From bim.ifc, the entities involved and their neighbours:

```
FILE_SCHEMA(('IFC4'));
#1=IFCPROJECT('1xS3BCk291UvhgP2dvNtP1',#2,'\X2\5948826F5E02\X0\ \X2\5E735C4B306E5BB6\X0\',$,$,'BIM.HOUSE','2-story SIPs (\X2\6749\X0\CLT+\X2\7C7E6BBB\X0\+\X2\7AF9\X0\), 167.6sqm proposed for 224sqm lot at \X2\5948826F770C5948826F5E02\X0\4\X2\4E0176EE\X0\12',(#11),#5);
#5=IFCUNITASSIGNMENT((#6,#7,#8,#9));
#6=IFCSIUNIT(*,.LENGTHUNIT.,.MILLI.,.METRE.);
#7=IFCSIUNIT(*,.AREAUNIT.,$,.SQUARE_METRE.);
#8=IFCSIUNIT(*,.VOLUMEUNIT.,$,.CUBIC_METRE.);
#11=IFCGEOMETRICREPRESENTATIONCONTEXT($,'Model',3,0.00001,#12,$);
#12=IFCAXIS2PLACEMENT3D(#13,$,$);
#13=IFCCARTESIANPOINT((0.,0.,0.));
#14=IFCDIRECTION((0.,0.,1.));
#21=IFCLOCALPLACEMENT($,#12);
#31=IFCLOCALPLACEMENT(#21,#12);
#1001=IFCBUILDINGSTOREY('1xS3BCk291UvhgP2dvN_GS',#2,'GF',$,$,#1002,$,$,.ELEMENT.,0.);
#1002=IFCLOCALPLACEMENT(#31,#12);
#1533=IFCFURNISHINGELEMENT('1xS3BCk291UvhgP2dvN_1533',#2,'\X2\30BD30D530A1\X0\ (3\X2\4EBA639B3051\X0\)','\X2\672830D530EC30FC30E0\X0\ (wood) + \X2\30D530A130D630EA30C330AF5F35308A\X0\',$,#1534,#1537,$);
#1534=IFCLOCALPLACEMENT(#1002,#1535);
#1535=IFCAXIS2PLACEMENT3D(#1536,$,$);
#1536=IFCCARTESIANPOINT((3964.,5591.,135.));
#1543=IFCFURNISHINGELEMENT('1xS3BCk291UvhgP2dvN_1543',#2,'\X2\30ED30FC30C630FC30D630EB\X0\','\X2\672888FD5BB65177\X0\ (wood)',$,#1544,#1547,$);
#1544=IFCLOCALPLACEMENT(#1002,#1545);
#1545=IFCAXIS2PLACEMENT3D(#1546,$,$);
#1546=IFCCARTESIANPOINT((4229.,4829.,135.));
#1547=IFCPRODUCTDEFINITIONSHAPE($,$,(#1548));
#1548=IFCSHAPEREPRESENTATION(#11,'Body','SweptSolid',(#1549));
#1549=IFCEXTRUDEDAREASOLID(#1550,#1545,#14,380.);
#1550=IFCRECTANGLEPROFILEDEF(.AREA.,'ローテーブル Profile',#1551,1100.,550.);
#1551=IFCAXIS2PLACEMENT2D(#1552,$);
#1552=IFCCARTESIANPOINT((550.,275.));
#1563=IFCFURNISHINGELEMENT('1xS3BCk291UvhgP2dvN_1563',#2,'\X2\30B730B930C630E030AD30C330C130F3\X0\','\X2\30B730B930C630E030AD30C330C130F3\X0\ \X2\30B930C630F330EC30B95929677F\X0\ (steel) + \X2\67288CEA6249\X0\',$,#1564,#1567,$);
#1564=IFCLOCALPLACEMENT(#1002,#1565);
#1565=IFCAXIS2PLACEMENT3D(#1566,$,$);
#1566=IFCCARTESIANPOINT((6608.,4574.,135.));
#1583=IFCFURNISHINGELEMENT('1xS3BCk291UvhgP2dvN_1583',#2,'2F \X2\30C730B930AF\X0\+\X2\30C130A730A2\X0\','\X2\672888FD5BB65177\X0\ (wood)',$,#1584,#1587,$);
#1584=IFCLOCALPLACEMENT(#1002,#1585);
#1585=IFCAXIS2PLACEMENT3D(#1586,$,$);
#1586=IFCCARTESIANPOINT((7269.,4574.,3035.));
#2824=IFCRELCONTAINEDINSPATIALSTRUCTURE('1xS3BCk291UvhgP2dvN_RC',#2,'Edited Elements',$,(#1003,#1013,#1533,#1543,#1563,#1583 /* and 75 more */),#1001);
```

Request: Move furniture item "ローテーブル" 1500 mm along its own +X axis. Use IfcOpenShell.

```python
import ifcopenshell
import ifcopenshell.api.geometry
import ifcopenshell.util.placement

model = ifcopenshell.open("bim.ifc")

item = model.by_guid("1xS3BCk291UvhgP2dvN_1543")
matrix = ifcopenshell.util.placement.get_local_placement(item.ObjectPlacement)
matrix[:3, 3] += matrix[:3, 0] * 1500.0
ifcopenshell.api.geometry.edit_object_placement(model, product=item, matrix=matrix, is_si=False)

print(ifcopenshell.util.placement.get_local_placement(item.ObjectPlacement).round(3) + 0.0)

model.write("bim_rev.ifc")
```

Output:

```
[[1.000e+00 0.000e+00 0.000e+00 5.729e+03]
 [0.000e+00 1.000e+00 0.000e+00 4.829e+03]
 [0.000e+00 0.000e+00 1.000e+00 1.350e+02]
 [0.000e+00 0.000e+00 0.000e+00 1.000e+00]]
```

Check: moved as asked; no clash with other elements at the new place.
